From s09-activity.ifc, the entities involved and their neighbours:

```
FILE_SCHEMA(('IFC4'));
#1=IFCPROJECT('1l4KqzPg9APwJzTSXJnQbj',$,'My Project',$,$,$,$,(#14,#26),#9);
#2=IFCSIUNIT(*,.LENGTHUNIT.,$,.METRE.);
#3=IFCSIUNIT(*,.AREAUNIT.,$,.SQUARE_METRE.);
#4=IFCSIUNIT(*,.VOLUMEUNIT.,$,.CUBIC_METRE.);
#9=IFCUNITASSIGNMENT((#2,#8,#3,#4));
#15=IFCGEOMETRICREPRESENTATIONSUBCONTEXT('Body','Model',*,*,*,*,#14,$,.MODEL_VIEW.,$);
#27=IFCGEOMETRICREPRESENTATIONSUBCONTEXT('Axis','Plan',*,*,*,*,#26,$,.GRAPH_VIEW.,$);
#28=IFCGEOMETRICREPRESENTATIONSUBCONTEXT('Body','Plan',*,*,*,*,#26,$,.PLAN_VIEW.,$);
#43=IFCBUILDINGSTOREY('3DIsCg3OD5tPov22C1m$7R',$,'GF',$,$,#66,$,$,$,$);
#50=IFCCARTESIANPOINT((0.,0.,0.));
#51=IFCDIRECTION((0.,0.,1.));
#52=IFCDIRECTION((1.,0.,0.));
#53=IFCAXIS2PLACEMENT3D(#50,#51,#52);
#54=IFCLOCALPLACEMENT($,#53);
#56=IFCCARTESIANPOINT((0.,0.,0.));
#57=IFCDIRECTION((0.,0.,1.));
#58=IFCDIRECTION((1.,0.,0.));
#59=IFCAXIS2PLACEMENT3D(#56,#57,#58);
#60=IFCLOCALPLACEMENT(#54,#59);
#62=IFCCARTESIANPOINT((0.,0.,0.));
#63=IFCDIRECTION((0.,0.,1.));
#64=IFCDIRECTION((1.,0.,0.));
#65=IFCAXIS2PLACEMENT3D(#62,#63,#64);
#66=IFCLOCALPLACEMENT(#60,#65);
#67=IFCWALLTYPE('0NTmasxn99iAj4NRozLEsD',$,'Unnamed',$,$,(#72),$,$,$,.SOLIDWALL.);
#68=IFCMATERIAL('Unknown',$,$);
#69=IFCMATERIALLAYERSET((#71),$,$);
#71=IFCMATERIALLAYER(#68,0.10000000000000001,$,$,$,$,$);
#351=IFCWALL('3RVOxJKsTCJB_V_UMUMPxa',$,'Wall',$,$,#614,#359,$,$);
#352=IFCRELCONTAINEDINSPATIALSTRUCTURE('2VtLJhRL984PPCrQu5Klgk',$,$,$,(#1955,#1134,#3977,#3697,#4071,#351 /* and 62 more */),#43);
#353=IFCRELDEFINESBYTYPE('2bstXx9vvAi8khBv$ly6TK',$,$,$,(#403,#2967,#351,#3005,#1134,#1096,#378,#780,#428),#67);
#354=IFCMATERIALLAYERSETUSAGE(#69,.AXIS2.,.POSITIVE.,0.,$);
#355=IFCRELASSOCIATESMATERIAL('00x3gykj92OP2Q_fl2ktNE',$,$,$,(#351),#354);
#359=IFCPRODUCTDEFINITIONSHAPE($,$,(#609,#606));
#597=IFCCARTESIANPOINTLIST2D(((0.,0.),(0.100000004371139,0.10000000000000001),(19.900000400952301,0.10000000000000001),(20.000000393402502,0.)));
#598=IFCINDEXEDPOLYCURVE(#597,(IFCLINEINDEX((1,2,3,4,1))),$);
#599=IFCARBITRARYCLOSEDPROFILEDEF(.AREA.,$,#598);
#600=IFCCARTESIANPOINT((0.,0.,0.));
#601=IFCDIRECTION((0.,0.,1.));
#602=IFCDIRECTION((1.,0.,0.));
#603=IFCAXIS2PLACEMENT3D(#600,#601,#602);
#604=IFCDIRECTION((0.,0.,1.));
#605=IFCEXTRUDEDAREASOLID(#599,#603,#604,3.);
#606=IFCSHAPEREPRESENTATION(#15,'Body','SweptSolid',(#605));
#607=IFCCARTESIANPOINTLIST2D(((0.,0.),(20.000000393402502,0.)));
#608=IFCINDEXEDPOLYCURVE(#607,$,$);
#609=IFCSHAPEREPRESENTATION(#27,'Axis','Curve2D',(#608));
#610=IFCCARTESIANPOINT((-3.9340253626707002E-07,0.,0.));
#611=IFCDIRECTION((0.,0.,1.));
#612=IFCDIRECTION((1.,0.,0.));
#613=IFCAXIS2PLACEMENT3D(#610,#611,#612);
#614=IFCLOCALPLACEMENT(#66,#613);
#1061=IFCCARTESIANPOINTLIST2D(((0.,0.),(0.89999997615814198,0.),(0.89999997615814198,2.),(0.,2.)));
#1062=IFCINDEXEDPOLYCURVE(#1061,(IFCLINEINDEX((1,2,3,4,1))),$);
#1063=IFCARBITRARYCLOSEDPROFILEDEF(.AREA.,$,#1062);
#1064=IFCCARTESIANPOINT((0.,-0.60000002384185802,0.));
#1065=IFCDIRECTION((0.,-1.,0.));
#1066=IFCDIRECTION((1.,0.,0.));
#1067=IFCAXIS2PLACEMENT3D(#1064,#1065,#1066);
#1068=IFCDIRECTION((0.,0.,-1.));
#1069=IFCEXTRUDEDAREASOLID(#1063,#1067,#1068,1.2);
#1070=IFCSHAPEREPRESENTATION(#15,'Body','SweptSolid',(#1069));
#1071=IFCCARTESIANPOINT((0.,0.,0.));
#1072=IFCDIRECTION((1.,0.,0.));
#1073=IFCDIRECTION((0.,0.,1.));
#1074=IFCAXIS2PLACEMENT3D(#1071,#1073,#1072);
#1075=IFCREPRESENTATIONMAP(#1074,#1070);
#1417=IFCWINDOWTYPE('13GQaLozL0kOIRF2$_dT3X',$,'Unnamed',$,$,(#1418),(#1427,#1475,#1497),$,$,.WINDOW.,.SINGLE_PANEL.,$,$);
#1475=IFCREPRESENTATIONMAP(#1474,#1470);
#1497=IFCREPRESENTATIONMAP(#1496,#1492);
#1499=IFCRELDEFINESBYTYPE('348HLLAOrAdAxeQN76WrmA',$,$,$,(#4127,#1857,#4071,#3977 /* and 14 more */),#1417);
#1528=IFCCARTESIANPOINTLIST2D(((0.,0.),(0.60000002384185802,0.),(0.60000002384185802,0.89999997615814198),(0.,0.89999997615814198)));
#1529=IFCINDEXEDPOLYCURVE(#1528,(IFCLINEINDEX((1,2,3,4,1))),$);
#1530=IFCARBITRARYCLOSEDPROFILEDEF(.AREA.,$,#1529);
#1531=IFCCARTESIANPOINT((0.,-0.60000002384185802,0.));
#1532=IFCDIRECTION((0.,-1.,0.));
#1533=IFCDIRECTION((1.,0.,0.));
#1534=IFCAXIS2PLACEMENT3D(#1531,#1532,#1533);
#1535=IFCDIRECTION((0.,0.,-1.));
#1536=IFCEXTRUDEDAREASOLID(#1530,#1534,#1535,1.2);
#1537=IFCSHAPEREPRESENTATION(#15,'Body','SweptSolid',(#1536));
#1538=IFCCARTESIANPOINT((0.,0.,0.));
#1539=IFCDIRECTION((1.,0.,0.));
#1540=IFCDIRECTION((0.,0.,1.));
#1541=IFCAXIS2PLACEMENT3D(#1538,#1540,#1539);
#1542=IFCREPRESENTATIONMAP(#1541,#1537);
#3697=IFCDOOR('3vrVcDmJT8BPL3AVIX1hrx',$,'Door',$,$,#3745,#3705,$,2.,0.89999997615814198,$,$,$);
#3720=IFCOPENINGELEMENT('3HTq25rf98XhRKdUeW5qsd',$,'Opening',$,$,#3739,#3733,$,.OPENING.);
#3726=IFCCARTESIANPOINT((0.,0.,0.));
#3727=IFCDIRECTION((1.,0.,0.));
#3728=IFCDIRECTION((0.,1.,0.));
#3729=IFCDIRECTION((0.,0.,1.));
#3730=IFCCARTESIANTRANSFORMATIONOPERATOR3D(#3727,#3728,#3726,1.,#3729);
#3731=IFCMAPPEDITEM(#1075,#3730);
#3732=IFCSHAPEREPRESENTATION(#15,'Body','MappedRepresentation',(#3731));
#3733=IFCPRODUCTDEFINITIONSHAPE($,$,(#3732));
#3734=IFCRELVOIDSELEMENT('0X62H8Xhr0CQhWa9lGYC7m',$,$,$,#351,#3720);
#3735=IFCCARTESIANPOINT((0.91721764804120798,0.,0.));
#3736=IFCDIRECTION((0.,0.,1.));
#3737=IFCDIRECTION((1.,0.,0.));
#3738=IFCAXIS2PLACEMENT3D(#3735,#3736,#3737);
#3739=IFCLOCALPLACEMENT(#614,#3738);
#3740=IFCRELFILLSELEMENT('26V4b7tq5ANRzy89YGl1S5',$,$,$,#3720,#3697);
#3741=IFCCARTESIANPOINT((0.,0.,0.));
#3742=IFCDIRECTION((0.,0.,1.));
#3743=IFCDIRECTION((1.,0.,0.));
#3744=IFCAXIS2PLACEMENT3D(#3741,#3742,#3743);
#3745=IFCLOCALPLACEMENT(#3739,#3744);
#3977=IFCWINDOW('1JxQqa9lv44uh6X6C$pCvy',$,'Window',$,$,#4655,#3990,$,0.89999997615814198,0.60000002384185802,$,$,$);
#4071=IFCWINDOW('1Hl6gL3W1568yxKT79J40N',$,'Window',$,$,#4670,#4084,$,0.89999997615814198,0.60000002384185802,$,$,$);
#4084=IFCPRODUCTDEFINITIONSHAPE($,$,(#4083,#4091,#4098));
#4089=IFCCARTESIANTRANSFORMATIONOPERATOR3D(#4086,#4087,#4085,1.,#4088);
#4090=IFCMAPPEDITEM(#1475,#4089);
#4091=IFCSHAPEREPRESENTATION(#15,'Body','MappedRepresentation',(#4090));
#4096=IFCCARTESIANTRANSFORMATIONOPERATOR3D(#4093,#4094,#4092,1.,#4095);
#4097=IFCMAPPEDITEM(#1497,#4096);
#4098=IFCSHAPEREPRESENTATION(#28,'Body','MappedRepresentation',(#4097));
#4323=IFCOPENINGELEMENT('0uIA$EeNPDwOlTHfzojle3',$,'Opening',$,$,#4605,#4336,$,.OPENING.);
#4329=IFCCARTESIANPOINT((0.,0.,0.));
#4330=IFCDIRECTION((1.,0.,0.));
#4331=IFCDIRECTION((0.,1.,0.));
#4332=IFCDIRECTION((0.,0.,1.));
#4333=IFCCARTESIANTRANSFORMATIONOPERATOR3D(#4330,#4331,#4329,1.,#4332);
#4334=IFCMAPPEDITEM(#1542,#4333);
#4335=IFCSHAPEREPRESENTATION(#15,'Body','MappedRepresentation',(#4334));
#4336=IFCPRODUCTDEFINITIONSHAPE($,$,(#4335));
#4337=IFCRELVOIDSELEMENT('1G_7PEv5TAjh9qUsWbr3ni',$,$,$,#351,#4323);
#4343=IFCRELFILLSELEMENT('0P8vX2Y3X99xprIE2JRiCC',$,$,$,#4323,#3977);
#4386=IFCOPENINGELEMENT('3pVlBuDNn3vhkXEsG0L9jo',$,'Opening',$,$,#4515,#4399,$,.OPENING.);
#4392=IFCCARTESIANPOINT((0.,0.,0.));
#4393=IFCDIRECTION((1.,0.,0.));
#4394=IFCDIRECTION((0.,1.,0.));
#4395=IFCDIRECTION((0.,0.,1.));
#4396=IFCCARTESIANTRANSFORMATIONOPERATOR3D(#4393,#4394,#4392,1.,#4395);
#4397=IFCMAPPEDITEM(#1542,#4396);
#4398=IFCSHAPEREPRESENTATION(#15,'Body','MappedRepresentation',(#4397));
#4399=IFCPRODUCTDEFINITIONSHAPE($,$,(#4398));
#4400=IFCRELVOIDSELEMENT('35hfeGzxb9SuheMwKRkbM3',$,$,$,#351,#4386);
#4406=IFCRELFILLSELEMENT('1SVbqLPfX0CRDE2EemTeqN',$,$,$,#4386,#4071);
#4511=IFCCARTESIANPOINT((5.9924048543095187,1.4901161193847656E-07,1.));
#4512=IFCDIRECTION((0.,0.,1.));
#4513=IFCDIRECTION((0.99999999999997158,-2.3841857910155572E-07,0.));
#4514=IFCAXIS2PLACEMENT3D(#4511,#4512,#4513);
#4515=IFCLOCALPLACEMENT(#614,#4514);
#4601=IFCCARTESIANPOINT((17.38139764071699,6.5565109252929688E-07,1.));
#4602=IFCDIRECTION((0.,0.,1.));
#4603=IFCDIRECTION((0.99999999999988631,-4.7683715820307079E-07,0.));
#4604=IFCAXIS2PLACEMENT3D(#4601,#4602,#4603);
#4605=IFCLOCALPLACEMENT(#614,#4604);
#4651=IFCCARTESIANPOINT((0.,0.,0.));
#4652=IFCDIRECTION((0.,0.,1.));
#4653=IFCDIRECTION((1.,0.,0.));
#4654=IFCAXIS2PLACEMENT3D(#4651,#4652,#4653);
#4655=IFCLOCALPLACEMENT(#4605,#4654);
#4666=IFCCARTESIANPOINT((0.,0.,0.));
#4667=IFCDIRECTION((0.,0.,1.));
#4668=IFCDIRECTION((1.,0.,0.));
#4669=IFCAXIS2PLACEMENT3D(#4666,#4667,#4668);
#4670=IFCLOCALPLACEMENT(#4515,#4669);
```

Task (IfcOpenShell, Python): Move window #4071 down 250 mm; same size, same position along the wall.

```python
import numpy as np
import ifcopenshell
import ifcopenshell.api.geometry
import ifcopenshell.util.placement
import ifcopenshell.util.unit

model = ifcopenshell.open("s09-activity.ifc")
unit_scale = ifcopenshell.util.unit.calculate_unit_scale(model)

window = model.by_id(4071)
opening = window.FillsVoids[0].RelatingOpeningElement
dz = -0.25 / unit_scale

shift = np.array([0.0, 0.0, dz])
# The window is placed relative to its opening, so it follows when the opening moves.
matrix = ifcopenshell.util.placement.get_local_placement(opening.ObjectPlacement)
matrix[:3, 3] += shift
ifcopenshell.api.geometry.edit_object_placement(
    model, product=opening, matrix=matrix, is_si=False, should_transform_children=True
)

print(f"moved by {dz * unit_scale:+.3f} m")

model.write("s09-activity_rev.ifc")
```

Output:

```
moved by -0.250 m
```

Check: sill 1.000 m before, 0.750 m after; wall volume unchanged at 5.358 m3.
